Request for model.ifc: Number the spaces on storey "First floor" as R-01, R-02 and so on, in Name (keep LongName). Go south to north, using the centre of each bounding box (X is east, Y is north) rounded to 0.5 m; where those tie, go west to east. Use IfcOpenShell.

First a look at what the model holds.

```python
import ifcopenshell
import ifcopenshell.util.element
import ifcopenshell.util.placement

model = ifcopenshell.open("model.ifc")
print(model.schema)
storey = next(s for s in model.by_type("IfcBuildingStorey") if s.Name == "First floor")
spaces = [e for e in ifcopenshell.util.element.get_decomposition(storey) if e.is_a("IfcSpace")]
for e in sorted(spaces, key=lambda e: e.id()):
    origin = ifcopenshell.util.placement.get_local_placement(e.ObjectPlacement)[:3, 3]
    print(e.id(), e.Name, e.LongName, origin.round(2) + 0.0, sep=" | ")
```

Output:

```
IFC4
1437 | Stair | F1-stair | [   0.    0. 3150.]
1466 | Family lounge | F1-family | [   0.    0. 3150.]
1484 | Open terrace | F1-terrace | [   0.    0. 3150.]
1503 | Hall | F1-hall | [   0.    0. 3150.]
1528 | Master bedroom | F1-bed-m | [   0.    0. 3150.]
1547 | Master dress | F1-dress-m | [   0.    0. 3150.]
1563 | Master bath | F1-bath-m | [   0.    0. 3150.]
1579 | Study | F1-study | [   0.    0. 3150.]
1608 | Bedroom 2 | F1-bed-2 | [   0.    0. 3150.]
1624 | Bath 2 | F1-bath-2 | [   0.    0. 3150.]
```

```python
import ifcopenshell
import ifcopenshell.geom
import ifcopenshell.util.element
import ifcopenshell.util.shape

model = ifcopenshell.open("model.ifc")
settings = ifcopenshell.geom.settings()
settings.set("use-world-coords", True)


def centre(element):
    shape = ifcopenshell.geom.create_shape(settings, element)
    return ifcopenshell.util.shape.get_bbox_centroid(shape.geometry)


storey = next(s for s in model.by_type("IfcBuildingStorey") if s.Name == "First floor")
spaces = [e for e in ifcopenshell.util.element.get_decomposition(storey) if e.is_a("IfcSpace")]

# Insertion points can sit at a corner or the storey origin, so sort by the geometry (in metres).
centres = {e: centre(e) for e in spaces}
spaces.sort(key=lambda e: (round(centres[e][1] / 0.5), centres[e][0]))

for i, e in enumerate(spaces, start=1):
    number = f"R-{i:02d}"
    e.Name = number
    print(e.id(), number)

model.write("model_rev.ifc")
```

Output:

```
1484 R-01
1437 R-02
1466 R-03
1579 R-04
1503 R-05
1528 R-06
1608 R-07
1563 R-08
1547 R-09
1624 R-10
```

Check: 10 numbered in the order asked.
